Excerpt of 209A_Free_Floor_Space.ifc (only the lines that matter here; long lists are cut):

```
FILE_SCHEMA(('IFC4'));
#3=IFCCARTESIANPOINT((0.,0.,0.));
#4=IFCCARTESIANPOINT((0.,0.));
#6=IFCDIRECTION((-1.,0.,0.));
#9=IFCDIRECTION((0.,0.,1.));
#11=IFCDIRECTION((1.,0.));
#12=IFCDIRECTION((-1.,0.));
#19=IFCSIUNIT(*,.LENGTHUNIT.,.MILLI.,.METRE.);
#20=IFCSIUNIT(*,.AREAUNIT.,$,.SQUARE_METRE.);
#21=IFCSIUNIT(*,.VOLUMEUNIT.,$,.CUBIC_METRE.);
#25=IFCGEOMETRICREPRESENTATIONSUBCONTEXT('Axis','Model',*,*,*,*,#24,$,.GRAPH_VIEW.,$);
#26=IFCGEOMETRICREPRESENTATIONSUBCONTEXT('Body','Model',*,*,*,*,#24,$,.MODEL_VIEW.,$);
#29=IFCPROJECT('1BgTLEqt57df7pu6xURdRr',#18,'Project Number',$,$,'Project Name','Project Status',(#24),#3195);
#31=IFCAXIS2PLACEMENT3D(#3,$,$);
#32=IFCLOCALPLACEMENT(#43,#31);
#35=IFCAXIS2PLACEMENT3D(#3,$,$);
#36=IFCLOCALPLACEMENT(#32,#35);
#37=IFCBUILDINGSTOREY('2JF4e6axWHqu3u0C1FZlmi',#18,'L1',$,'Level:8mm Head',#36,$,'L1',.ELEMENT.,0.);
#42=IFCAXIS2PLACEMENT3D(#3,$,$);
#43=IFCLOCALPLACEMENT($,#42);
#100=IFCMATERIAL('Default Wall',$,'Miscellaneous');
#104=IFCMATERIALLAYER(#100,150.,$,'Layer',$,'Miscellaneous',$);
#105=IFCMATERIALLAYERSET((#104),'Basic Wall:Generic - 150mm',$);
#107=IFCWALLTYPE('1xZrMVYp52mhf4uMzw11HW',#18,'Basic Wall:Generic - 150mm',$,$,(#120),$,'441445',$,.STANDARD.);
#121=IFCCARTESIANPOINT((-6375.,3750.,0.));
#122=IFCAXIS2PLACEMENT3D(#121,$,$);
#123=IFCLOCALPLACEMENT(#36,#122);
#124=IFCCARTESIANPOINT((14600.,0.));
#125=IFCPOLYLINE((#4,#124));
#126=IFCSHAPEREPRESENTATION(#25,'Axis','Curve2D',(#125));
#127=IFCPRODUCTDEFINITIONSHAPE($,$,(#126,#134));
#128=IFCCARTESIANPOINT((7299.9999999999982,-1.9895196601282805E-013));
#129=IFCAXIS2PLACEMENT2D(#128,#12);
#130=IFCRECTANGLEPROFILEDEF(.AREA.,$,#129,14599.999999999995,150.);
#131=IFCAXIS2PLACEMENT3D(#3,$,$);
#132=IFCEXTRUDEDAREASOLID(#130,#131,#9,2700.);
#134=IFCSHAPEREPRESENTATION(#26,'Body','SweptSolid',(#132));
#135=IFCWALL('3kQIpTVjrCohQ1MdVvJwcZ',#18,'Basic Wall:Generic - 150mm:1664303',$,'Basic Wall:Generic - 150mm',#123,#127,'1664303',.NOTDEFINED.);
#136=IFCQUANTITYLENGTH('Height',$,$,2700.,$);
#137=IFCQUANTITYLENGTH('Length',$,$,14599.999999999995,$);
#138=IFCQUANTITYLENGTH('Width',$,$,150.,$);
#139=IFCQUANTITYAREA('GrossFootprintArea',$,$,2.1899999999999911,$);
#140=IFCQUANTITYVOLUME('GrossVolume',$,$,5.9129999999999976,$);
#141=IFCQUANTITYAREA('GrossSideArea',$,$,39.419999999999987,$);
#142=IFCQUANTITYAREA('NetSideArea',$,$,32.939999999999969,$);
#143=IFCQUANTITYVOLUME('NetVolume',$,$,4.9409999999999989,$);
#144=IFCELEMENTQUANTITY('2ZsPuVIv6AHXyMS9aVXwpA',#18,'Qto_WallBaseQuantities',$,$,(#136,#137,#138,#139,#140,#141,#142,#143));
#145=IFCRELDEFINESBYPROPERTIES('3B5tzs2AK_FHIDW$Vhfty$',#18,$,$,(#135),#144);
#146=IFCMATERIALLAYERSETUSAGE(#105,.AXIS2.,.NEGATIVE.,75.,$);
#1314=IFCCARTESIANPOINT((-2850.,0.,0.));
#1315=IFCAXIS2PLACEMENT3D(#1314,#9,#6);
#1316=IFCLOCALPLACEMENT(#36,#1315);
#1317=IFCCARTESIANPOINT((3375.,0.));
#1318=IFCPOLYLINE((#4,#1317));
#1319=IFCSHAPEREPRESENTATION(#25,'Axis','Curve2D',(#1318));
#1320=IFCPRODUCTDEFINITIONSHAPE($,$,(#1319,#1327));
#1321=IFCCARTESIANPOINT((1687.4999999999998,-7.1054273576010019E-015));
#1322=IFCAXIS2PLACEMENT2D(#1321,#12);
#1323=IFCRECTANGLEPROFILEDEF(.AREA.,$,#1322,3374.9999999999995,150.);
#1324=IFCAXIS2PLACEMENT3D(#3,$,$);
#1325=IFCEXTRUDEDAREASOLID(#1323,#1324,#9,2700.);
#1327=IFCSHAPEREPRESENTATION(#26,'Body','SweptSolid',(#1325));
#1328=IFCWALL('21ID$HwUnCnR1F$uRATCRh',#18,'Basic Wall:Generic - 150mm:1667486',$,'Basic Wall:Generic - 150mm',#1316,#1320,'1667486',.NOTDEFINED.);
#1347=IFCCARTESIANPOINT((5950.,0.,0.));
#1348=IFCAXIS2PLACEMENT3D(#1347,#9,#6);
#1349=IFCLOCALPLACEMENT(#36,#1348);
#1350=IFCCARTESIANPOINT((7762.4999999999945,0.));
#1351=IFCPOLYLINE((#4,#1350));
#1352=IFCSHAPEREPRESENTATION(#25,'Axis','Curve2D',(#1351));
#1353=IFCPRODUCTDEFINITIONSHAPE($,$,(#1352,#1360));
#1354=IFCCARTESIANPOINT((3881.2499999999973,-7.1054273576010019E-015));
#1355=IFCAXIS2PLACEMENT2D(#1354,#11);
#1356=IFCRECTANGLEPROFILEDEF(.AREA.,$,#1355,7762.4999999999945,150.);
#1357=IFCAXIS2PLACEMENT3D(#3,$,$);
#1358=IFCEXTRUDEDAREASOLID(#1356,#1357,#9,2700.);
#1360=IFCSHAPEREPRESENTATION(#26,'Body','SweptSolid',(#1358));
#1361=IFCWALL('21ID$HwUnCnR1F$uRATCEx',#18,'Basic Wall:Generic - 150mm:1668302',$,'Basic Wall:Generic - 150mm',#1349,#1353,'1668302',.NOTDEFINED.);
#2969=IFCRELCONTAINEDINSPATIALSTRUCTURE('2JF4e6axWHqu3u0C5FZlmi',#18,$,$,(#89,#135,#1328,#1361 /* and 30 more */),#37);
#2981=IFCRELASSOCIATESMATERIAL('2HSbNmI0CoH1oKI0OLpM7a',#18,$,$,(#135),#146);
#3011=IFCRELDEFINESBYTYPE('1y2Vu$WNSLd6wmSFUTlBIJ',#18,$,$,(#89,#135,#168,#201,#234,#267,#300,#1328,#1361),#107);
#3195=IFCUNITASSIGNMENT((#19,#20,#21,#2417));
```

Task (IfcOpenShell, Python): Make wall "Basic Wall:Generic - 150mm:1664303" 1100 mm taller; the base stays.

```python
import ifcopenshell
import ifcopenshell.api.pset
import ifcopenshell.geom
import ifcopenshell.util.element
import ifcopenshell.util.representation
import ifcopenshell.util.shape
import ifcopenshell.util.unit

model = ifcopenshell.open("209A_Free_Floor_Space.ifc")
unit_scale = ifcopenshell.util.unit.calculate_unit_scale(model)
area_scale = ifcopenshell.util.unit.calculate_unit_scale(model, "AREAUNIT")
volume_scale = ifcopenshell.util.unit.calculate_unit_scale(model, "VOLUMEUNIT")
settings = ifcopenshell.geom.settings()


def volume(element):
    """Net volume in cubic metres, openings subtracted."""
    shape = ifcopenshell.geom.create_shape(settings, element)
    return ifcopenshell.util.shape.get_volume(shape.geometry)


wall = model.by_guid("3kQIpTVjrCohQ1MdVvJwcZ")
before = volume(wall)

body = ifcopenshell.util.representation.get_representation(wall, "Model", "Body")
solid = body.Items[0]
old_height = solid.Depth
solid.Depth += 1100.0
after = volume(wall)
thickness = 0.15  # wall thickness in metres

# Update the stored height, areas and volumes.
qto = model.by_id(ifcopenshell.util.element.get_pset(wall, "Qto_WallBaseQuantities", should_inherit=False)["id"])
ifcopenshell.api.pset.edit_qto(model, qto=qto, properties={
    "Height": solid.Depth,
    "GrossVolume": ifcopenshell.util.element.get_pset(wall, "Qto_WallBaseQuantities", "GrossVolume") * solid.Depth / old_height,
    "GrossSideArea": ifcopenshell.util.element.get_pset(wall, "Qto_WallBaseQuantities", "GrossSideArea") * solid.Depth / old_height,
    "NetSideArea": after / thickness / area_scale,
    "NetVolume": after / volume_scale,
})

print(f"height {old_height:g} -> {solid.Depth:g}, volume {before:.3f} -> {after:.3f} m3")

model.write("209A_Free_Floor_Space_v2.ifc")
```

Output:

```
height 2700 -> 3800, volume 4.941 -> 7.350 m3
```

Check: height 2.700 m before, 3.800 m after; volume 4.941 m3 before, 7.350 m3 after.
